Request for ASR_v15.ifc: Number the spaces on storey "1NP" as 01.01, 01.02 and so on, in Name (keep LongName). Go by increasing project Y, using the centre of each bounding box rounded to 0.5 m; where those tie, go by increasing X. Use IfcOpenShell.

First a look at what the model holds.

```python
import ifcopenshell
import ifcopenshell.util.element
import ifcopenshell.util.placement

model = ifcopenshell.open("ASR_v15.ifc")
print(model.schema)
storey = next(s for s in model.by_type("IfcBuildingStorey") if s.Name == "1NP")
spaces = [e for e in ifcopenshell.util.element.get_decomposition(storey) if e.is_a("IfcSpace")]
for e in sorted(spaces, key=lambda e: e.id()):
    origin = ifcopenshell.util.placement.get_local_placement(e.ObjectPlacement)[:3, 3]
    print(e.id(), e.Name, e.LongName, origin.round(2) + 0.0, sep=" | ")
```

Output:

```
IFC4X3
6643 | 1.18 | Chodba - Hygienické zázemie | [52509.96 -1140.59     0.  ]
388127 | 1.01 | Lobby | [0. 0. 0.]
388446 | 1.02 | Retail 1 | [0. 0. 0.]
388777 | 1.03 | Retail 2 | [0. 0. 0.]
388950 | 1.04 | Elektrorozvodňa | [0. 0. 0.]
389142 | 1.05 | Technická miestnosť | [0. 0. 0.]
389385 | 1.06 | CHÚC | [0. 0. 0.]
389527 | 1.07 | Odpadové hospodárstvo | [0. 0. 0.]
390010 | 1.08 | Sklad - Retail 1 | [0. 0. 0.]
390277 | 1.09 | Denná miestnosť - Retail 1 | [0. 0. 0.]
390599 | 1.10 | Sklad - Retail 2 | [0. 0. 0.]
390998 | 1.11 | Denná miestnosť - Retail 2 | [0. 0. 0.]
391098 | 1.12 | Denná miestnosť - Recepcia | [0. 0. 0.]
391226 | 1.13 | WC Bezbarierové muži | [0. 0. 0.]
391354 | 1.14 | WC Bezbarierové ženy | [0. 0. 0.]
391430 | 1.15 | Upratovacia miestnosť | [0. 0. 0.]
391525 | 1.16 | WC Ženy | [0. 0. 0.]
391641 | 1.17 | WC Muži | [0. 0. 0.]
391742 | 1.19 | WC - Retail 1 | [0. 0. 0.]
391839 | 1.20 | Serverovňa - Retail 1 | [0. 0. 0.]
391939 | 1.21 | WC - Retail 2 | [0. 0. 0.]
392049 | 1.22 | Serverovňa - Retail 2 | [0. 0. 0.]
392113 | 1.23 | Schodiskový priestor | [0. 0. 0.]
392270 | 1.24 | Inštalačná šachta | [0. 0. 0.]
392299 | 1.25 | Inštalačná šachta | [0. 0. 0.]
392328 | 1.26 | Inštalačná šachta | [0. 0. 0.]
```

```python
import ifcopenshell
import ifcopenshell.geom
import ifcopenshell.util.element
import ifcopenshell.util.shape

model = ifcopenshell.open("ASR_v15.ifc")
settings = ifcopenshell.geom.settings()
settings.set("use-world-coords", True)


def centre(element):
    shape = ifcopenshell.geom.create_shape(settings, element)
    return ifcopenshell.util.shape.get_bbox_centroid(shape.geometry)


storey = next(s for s in model.by_type("IfcBuildingStorey") if s.Name == "1NP")
spaces = [e for e in ifcopenshell.util.element.get_decomposition(storey) if e.is_a("IfcSpace")]

# Insertion points can sit at a corner or the storey origin, so sort by the geometry (in metres).
centres = {e: centre(e) for e in spaces}
spaces.sort(key=lambda e: (round(centres[e][1] / 0.5), centres[e][0]))

for i, e in enumerate(spaces, start=1):
    number = f"01.{i:02d}"
    e.Name = number
    print(e.id(), number)

model.write("ASR_v15_v2.ifc")
```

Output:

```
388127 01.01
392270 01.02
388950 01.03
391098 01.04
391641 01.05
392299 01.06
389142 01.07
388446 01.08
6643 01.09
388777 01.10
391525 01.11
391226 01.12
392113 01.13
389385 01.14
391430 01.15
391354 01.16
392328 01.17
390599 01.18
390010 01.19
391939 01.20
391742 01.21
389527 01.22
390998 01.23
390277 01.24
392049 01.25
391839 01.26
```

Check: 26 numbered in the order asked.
